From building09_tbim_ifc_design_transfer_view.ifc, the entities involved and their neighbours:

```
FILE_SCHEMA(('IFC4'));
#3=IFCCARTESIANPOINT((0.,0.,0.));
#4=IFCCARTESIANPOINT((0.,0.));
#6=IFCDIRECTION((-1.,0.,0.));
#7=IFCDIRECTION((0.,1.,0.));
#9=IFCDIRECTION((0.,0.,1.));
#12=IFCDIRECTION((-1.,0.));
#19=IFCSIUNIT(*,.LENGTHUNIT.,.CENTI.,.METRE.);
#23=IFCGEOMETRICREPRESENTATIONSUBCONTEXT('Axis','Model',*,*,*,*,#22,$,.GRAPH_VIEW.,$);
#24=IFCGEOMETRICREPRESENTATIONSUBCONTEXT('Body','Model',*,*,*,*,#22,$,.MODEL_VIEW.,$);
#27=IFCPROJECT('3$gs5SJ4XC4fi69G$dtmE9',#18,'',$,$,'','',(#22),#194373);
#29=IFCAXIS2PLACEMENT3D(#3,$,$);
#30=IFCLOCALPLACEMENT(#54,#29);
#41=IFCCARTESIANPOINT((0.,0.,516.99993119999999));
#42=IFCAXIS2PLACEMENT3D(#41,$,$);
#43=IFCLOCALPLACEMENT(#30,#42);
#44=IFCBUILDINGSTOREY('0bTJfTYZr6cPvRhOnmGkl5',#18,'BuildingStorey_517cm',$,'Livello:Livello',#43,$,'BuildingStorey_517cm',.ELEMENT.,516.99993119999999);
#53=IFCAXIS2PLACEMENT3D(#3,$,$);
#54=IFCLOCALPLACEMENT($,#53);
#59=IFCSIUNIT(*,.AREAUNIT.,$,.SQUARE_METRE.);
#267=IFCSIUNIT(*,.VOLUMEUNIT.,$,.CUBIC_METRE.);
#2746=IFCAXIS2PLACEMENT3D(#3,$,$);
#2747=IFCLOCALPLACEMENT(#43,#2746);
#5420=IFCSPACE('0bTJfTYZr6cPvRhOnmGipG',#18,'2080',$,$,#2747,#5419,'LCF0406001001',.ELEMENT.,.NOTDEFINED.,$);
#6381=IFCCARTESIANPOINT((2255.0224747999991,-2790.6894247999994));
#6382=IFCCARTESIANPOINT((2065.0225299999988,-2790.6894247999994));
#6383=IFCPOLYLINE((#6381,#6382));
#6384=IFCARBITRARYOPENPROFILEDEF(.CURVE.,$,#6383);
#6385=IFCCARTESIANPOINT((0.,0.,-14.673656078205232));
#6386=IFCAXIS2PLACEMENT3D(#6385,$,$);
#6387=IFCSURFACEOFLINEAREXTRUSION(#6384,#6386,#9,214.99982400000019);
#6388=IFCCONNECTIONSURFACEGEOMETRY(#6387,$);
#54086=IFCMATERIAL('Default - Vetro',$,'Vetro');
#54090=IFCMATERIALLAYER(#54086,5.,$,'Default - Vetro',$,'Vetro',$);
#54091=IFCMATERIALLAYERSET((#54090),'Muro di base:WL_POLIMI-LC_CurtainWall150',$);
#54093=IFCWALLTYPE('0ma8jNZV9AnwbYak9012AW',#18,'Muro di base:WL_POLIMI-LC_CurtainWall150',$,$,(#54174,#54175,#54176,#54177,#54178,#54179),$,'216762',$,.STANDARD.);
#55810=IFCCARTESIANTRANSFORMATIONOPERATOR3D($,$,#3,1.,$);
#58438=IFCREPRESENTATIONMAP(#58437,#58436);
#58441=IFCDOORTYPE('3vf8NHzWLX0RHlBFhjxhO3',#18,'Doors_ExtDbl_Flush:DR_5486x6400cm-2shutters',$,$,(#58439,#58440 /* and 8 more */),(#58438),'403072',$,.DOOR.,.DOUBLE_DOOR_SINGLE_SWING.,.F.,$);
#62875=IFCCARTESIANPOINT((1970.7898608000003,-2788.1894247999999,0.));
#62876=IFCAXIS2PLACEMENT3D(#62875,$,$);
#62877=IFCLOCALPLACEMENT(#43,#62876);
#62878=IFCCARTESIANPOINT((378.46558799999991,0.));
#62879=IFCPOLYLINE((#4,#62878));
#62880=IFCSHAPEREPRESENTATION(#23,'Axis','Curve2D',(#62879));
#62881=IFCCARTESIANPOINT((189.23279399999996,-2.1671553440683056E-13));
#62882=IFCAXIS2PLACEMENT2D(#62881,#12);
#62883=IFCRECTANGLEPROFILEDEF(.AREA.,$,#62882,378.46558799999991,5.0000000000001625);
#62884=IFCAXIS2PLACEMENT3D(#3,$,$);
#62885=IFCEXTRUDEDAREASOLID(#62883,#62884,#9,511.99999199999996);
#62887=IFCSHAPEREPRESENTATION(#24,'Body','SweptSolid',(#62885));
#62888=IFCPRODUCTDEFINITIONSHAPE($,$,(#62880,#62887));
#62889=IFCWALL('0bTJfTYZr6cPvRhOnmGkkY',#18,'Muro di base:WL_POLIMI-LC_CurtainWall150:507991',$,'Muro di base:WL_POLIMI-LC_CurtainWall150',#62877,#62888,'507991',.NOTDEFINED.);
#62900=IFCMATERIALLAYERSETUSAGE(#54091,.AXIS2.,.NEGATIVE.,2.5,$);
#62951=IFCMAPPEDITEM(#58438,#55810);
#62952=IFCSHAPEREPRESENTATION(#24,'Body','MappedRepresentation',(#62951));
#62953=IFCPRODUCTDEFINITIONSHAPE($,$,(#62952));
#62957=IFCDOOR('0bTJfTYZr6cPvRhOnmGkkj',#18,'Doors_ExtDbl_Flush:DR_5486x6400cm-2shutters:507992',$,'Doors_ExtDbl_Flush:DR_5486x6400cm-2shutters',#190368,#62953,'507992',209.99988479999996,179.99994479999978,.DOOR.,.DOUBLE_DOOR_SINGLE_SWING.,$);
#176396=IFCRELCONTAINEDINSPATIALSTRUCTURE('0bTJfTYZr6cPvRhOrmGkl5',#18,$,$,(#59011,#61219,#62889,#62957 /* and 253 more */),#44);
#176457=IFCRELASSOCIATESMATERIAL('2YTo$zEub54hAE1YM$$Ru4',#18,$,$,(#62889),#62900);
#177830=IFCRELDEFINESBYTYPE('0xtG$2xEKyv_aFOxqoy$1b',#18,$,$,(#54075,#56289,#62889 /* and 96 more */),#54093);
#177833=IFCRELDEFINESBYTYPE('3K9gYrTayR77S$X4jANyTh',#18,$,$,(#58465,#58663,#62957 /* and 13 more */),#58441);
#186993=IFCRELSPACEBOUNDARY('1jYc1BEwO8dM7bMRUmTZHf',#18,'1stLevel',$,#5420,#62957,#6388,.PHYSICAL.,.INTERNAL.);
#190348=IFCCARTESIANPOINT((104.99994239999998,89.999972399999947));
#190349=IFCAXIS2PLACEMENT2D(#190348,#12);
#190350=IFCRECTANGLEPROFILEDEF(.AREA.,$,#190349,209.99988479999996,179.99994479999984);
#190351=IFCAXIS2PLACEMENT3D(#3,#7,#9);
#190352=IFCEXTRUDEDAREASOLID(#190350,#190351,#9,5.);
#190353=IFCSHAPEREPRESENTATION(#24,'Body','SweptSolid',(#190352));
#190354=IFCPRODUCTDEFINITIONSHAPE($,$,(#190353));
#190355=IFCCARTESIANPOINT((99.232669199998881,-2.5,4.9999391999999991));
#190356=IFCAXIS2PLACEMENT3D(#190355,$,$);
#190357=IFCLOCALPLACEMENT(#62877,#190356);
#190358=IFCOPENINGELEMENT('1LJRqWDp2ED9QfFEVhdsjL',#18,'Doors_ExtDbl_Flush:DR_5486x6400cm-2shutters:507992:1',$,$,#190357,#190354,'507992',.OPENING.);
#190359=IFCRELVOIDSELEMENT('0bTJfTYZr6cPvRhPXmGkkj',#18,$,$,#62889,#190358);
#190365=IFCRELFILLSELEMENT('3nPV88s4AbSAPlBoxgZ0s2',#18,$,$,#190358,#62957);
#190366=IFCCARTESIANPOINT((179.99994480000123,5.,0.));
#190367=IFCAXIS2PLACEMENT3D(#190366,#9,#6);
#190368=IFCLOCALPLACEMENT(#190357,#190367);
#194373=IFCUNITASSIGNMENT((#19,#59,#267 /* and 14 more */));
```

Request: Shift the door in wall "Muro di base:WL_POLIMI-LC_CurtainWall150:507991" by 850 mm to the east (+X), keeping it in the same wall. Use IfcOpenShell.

```python
import numpy as np
import ifcopenshell
import ifcopenshell.api.geometry
import ifcopenshell.util.placement
import ifcopenshell.util.unit

model = ifcopenshell.open("building09_tbim_ifc_design_transfer_view.ifc")
unit_scale = ifcopenshell.util.unit.calculate_unit_scale(model)

door = model.by_guid("0bTJfTYZr6cPvRhOnmGkkj")
opening = door.FillsVoids[0].RelatingOpeningElement
wall = opening.VoidsElements[0].RelatingBuildingElement

wall_matrix = ifcopenshell.util.placement.get_local_placement(wall.ObjectPlacement)
shift = wall_matrix[:3, 0] * 0.85 / unit_scale
before = ifcopenshell.util.placement.get_local_placement(door.ObjectPlacement)[:3, 3].copy()

# The door is placed relative to its opening, so it follows when the opening moves.
matrix = ifcopenshell.util.placement.get_local_placement(opening.ObjectPlacement)
matrix[:3, 3] += shift
ifcopenshell.api.geometry.edit_object_placement(
    model, product=opening, matrix=matrix, is_si=False, should_transform_children=True
)

# Space boundary surfaces are stored in each space's coordinates; move them too.
for rel in door.ProvidesBoundaries:
    if not rel.ConnectionGeometry:
        continue
    surface = rel.ConnectionGeometry.SurfaceOnRelatingElement
    space_matrix = ifcopenshell.util.placement.get_local_placement(rel.RelatingSpace.ObjectPlacement)
    point = np.array(surface.Position.Location.Coordinates) + space_matrix[:3, :3].T @ shift
    surface.Position = model.createIfcAxis2Placement3D(
        model.createIfcCartesianPoint(point.tolist()), surface.Position.Axis, surface.Position.RefDirection
    )

after = ifcopenshell.util.placement.get_local_placement(door.ObjectPlacement)[:3, 3]
print("door moved by", (after - before).round(3) + 0.0)

model.write("building09_tbim_ifc_design_transfer_view_v2.ifc")
```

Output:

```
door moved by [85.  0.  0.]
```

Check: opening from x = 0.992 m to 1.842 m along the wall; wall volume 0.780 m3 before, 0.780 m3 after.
